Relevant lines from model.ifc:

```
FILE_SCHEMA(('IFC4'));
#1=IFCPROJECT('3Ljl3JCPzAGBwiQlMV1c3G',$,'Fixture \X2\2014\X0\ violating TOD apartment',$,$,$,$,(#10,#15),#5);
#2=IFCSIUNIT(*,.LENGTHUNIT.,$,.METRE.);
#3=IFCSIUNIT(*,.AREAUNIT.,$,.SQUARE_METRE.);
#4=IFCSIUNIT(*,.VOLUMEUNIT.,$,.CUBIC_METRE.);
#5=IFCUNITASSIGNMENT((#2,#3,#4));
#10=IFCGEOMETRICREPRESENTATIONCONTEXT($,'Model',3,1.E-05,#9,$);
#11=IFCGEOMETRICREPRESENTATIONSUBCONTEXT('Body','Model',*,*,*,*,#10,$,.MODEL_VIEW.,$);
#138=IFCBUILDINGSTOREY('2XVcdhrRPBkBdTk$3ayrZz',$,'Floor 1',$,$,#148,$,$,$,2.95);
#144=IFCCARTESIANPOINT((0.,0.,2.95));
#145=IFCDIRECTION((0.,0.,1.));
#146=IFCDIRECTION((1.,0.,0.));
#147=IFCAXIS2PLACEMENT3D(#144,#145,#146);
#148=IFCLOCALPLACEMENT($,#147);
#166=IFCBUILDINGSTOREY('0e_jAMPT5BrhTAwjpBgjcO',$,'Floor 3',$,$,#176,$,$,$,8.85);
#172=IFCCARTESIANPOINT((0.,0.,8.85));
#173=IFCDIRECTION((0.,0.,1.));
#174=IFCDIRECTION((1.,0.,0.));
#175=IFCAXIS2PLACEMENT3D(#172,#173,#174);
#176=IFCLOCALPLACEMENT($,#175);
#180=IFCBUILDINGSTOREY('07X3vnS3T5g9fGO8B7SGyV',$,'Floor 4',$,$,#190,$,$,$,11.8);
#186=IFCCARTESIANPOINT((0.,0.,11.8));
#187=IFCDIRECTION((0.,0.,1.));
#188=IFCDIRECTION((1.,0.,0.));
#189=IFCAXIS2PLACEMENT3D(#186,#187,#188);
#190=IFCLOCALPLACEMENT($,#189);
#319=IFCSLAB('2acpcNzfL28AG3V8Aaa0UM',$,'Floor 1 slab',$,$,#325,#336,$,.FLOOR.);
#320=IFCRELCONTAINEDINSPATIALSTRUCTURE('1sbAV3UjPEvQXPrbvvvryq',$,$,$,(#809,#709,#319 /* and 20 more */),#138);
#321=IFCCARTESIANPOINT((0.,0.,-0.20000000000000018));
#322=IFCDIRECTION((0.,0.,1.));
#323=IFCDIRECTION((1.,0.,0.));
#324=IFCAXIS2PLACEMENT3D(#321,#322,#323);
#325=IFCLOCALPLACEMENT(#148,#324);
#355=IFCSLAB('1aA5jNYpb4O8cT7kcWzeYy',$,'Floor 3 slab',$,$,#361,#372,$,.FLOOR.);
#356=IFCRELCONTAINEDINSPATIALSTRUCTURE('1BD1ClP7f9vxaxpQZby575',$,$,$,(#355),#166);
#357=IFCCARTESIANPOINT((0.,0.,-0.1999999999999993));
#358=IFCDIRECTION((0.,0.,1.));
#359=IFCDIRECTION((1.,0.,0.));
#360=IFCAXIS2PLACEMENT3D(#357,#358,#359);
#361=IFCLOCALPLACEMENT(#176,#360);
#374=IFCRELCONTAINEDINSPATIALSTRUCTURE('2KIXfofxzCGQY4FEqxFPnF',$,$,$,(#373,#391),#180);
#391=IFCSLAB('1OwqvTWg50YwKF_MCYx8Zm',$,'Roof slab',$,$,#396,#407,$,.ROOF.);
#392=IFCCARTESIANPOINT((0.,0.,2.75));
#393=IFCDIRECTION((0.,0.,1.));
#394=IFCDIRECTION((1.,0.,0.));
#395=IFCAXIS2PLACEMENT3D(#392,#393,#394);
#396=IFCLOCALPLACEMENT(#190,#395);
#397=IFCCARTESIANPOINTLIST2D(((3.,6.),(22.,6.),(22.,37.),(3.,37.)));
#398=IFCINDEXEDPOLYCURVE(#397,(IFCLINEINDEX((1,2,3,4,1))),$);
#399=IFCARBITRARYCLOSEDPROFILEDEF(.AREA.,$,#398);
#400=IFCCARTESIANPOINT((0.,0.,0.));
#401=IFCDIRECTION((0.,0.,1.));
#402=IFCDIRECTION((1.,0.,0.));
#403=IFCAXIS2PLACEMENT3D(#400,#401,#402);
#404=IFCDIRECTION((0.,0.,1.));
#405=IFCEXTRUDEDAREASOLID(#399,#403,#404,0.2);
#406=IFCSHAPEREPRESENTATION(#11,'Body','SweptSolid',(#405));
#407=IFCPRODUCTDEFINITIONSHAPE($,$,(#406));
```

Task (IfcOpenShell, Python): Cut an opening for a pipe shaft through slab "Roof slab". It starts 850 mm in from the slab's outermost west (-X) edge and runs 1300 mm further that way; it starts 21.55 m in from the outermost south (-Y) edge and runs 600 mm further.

```python
import numpy as np
import ifcopenshell
import ifcopenshell.api.feature
import ifcopenshell.api.geometry
import ifcopenshell.api.root
import ifcopenshell.geom
import ifcopenshell.util.placement
import ifcopenshell.util.representation
import ifcopenshell.util.shape
import ifcopenshell.util.unit

model = ifcopenshell.open("model.ifc")
unit_scale = ifcopenshell.util.unit.calculate_unit_scale(model)
settings = ifcopenshell.geom.settings()


def volume(element):
    """Net volume in cubic metres, openings subtracted."""
    shape = ifcopenshell.geom.create_shape(settings, element)
    return ifcopenshell.util.shape.get_volume(shape.geometry)


slab = model.by_guid("1OwqvTWg50YwKF_MCYx8Zm")
before = volume(slab)

# Extent in the slab's own axes, in metres. The edges named are its -X and -Y sides.
slab_shape = ifcopenshell.geom.create_shape(settings, slab)
vertices = ifcopenshell.util.shape.get_vertices(slab_shape.geometry)
x_min, y_min, bottom = vertices.min(axis=0)
top = vertices[:, 2].max()

opening = ifcopenshell.api.root.create_entity(model, ifc_class="IfcOpeningElement", name="Pipe shaft opening", predefined_type="OPENING")
context = ifcopenshell.util.representation.get_context(model, "Model", "Body", "MODEL_VIEW")
width, depth = 1.3, 0.6
outline = [(0.0, 0.0), (width, 0.0), (width, depth), (0.0, depth), (0.0, 0.0)]
# Overshoot both faces by 50 mm so the cut is clean.
shape = ifcopenshell.api.geometry.add_slab_representation(
    model, context=context, depth=top - bottom + 0.1, polyline=outline
)
ifcopenshell.api.geometry.assign_representation(model, product=opening, representation=shape)

matrix = ifcopenshell.util.placement.get_local_placement(slab.ObjectPlacement)
matrix[:, 3] = matrix @ np.append(np.array([x_min + 0.85, y_min + 21.55, bottom - 0.05]) / unit_scale, 1.0)
ifcopenshell.api.geometry.edit_object_placement(model, product=opening, matrix=matrix, is_si=False)
ifcopenshell.api.feature.add_feature(model, feature=opening, element=slab)

after = volume(slab)

print(f"slab volume {before:.3f} -> {after:.3f} m3")

model.write("model_v2.ifc")
```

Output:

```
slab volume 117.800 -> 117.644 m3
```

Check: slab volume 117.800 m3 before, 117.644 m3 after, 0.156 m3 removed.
